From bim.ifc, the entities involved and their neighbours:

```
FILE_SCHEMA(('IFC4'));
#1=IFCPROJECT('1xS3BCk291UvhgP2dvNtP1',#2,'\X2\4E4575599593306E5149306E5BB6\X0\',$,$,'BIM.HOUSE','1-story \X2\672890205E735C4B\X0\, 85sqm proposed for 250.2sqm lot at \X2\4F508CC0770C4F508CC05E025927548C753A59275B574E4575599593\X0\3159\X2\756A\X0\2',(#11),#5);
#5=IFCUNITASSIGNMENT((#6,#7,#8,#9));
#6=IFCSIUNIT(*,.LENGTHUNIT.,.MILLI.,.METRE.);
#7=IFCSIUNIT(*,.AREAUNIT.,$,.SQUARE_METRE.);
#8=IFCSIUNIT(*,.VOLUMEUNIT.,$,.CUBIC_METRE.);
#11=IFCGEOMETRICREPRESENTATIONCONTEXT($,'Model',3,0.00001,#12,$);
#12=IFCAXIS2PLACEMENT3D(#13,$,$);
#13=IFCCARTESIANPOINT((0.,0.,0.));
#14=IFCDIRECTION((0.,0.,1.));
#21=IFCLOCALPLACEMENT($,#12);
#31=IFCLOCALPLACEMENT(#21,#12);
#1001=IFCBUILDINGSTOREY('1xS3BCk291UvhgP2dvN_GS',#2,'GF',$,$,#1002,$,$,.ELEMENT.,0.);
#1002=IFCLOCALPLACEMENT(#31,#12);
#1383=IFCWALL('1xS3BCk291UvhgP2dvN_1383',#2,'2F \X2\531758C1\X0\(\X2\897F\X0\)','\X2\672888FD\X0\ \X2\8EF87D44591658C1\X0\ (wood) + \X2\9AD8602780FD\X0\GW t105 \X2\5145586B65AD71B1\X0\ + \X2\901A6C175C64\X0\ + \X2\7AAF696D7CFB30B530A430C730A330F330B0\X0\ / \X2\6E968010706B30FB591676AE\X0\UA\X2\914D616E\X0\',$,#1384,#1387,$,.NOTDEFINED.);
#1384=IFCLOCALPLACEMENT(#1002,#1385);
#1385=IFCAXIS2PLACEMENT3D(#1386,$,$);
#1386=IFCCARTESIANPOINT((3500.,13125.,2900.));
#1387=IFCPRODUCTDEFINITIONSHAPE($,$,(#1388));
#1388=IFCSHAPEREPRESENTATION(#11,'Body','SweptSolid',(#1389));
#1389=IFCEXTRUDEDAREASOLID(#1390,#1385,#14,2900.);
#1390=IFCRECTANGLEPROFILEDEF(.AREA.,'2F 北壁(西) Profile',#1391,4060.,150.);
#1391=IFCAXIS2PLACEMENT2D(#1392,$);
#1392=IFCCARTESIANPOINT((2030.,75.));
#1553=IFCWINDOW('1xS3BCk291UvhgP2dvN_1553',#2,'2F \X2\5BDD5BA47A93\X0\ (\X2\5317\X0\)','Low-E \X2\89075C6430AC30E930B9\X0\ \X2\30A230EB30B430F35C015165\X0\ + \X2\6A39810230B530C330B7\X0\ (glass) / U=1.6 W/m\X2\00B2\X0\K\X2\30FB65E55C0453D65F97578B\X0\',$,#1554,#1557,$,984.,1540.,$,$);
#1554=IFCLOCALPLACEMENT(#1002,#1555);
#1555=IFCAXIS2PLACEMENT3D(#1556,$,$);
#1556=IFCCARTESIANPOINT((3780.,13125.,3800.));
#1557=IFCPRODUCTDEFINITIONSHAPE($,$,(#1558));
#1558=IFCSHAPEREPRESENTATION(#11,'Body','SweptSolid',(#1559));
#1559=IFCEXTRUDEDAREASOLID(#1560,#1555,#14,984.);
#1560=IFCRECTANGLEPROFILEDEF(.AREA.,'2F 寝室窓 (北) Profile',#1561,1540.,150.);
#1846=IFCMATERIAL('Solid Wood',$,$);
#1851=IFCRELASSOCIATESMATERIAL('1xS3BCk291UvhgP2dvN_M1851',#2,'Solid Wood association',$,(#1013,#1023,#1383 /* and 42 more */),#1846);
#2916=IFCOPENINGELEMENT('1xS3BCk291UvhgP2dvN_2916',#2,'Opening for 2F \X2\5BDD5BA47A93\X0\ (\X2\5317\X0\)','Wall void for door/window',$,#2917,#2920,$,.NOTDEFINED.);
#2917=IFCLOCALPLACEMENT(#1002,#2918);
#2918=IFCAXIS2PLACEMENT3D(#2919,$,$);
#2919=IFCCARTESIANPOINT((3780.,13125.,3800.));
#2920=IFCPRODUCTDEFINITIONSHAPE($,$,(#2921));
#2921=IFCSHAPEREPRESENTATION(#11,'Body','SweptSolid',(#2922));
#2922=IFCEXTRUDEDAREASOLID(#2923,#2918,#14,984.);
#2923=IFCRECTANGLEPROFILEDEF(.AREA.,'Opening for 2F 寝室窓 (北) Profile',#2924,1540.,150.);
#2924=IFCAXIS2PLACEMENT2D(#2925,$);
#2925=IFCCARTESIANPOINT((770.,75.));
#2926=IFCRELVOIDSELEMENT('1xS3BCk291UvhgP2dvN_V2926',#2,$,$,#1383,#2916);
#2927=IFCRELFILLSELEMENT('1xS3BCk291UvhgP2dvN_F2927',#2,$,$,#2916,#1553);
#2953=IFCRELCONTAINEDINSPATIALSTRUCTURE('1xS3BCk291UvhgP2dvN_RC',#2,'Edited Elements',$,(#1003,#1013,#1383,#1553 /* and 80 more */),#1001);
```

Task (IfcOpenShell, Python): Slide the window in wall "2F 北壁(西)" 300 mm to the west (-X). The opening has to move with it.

```python
import ifcopenshell
import ifcopenshell.api.geometry
import ifcopenshell.util.placement

model = ifcopenshell.open("bim.ifc")

window = model.by_guid("1xS3BCk291UvhgP2dvN_1553")
opening = window.FillsVoids[0].RelatingOpeningElement
wall = opening.VoidsElements[0].RelatingBuildingElement

wall_matrix = ifcopenshell.util.placement.get_local_placement(wall.ObjectPlacement)
shift = wall_matrix[:3, 0] * -300.0
before = ifcopenshell.util.placement.get_local_placement(window.ObjectPlacement)[:3, 3].copy()

# The window is not placed relative to its opening, so move both.
for product in (opening, window):
    matrix = ifcopenshell.util.placement.get_local_placement(product.ObjectPlacement)
    matrix[:3, 3] += shift
    ifcopenshell.api.geometry.edit_object_placement(model, product=product, matrix=matrix, is_si=False)

after = ifcopenshell.util.placement.get_local_placement(window.ObjectPlacement)[:3, 3]
print("window moved by", (after - before).round(3) + 0.0)

model.write("bim_v2.ifc")
```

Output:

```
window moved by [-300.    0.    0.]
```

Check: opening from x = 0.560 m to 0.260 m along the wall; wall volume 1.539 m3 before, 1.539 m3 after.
